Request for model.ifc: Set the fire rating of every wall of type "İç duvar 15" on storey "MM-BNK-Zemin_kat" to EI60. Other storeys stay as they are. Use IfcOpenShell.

First a look at what the model holds.

```python
import ifcopenshell
import ifcopenshell.util.element

model = ifcopenshell.open("model.ifc")
print(model.schema)
storey = next(s for s in model.by_type("IfcBuildingStorey") if s.Name == "MM-BNK-Zemin_kat")
walls = [e for e in ifcopenshell.util.element.get_decomposition(storey) if e.is_a("IfcWall")]
seen = {}
for e in walls:
    element_type = ifcopenshell.util.element.get_type(e)
    key = (element_type.Name if element_type != e and element_type else None, ifcopenshell.util.element.get_pset(e, "Pset_WallCommon", "FireRating"))
    seen[key] = seen.get(key, 0) + 1
for (name, value), count in sorted(seen.items(), key=str):
    print(count, "x", name, "|", value)
```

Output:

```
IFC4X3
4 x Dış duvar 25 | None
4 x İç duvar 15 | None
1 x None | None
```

```python
import ifcopenshell
import ifcopenshell.api.pset
import ifcopenshell.util.element

model = ifcopenshell.open("model.ifc")

storey = next(s for s in model.by_type("IfcBuildingStorey") if s.Name == "MM-BNK-Zemin_kat")
walls = [e for e in ifcopenshell.util.element.get_decomposition(storey) if e.is_a("IfcWall")]

count = 0
for e in walls:
    element_type = ifcopenshell.util.element.get_type(e)
    if element_type in (None, e) or element_type.Name != "İç duvar 15":
        continue
    # add_pset returns the element's existing set when there is one.
    pset = ifcopenshell.api.pset.add_pset(model, product=e, name="Pset_WallCommon")
    ifcopenshell.api.pset.edit_pset(model, pset=pset, properties={"FireRating": "EI60"})
    count += 1

print(count, "walls updated")

model.write("model_edited.ifc")
```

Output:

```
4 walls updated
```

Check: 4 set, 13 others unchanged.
